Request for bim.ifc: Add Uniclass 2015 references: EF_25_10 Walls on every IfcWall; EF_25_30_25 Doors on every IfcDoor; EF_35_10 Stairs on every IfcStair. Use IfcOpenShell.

First a look at what the model holds.

```python
import ifcopenshell

model = ifcopenshell.open("bim.ifc")
print(model.schema)
print("classifications:", [c.Name for c in model.by_type("IfcClassification")])
for ifc_class in ("IfcDoor", "IfcRoof", "IfcStair", "IfcWall", "IfcWindow"):
    print(ifc_class, len(model.by_type(ifc_class)))
```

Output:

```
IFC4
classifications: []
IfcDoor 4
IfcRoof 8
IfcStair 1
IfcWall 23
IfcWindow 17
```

```python
import ifcopenshell
import ifcopenshell.api.classification

model = ifcopenshell.open("bim.ifc")

system = ifcopenshell.api.classification.add_classification(model, classification="Uniclass 2015")

codes = {
    "IfcWall": ("EF_25_10", "Walls"),
    "IfcDoor": ("EF_25_30_25", "Doors"),
    "IfcStair": ("EF_35_10", "Stairs"),
}
for ifc_class, (code, name) in codes.items():
    products = model.by_type(ifc_class)
    ifcopenshell.api.classification.add_reference(
        model, products=products, classification=system, identification=code, name=name
    )
    print(code, len(products))

model.write("bim_v2.ifc")
```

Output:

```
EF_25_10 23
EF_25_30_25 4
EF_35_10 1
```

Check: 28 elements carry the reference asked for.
